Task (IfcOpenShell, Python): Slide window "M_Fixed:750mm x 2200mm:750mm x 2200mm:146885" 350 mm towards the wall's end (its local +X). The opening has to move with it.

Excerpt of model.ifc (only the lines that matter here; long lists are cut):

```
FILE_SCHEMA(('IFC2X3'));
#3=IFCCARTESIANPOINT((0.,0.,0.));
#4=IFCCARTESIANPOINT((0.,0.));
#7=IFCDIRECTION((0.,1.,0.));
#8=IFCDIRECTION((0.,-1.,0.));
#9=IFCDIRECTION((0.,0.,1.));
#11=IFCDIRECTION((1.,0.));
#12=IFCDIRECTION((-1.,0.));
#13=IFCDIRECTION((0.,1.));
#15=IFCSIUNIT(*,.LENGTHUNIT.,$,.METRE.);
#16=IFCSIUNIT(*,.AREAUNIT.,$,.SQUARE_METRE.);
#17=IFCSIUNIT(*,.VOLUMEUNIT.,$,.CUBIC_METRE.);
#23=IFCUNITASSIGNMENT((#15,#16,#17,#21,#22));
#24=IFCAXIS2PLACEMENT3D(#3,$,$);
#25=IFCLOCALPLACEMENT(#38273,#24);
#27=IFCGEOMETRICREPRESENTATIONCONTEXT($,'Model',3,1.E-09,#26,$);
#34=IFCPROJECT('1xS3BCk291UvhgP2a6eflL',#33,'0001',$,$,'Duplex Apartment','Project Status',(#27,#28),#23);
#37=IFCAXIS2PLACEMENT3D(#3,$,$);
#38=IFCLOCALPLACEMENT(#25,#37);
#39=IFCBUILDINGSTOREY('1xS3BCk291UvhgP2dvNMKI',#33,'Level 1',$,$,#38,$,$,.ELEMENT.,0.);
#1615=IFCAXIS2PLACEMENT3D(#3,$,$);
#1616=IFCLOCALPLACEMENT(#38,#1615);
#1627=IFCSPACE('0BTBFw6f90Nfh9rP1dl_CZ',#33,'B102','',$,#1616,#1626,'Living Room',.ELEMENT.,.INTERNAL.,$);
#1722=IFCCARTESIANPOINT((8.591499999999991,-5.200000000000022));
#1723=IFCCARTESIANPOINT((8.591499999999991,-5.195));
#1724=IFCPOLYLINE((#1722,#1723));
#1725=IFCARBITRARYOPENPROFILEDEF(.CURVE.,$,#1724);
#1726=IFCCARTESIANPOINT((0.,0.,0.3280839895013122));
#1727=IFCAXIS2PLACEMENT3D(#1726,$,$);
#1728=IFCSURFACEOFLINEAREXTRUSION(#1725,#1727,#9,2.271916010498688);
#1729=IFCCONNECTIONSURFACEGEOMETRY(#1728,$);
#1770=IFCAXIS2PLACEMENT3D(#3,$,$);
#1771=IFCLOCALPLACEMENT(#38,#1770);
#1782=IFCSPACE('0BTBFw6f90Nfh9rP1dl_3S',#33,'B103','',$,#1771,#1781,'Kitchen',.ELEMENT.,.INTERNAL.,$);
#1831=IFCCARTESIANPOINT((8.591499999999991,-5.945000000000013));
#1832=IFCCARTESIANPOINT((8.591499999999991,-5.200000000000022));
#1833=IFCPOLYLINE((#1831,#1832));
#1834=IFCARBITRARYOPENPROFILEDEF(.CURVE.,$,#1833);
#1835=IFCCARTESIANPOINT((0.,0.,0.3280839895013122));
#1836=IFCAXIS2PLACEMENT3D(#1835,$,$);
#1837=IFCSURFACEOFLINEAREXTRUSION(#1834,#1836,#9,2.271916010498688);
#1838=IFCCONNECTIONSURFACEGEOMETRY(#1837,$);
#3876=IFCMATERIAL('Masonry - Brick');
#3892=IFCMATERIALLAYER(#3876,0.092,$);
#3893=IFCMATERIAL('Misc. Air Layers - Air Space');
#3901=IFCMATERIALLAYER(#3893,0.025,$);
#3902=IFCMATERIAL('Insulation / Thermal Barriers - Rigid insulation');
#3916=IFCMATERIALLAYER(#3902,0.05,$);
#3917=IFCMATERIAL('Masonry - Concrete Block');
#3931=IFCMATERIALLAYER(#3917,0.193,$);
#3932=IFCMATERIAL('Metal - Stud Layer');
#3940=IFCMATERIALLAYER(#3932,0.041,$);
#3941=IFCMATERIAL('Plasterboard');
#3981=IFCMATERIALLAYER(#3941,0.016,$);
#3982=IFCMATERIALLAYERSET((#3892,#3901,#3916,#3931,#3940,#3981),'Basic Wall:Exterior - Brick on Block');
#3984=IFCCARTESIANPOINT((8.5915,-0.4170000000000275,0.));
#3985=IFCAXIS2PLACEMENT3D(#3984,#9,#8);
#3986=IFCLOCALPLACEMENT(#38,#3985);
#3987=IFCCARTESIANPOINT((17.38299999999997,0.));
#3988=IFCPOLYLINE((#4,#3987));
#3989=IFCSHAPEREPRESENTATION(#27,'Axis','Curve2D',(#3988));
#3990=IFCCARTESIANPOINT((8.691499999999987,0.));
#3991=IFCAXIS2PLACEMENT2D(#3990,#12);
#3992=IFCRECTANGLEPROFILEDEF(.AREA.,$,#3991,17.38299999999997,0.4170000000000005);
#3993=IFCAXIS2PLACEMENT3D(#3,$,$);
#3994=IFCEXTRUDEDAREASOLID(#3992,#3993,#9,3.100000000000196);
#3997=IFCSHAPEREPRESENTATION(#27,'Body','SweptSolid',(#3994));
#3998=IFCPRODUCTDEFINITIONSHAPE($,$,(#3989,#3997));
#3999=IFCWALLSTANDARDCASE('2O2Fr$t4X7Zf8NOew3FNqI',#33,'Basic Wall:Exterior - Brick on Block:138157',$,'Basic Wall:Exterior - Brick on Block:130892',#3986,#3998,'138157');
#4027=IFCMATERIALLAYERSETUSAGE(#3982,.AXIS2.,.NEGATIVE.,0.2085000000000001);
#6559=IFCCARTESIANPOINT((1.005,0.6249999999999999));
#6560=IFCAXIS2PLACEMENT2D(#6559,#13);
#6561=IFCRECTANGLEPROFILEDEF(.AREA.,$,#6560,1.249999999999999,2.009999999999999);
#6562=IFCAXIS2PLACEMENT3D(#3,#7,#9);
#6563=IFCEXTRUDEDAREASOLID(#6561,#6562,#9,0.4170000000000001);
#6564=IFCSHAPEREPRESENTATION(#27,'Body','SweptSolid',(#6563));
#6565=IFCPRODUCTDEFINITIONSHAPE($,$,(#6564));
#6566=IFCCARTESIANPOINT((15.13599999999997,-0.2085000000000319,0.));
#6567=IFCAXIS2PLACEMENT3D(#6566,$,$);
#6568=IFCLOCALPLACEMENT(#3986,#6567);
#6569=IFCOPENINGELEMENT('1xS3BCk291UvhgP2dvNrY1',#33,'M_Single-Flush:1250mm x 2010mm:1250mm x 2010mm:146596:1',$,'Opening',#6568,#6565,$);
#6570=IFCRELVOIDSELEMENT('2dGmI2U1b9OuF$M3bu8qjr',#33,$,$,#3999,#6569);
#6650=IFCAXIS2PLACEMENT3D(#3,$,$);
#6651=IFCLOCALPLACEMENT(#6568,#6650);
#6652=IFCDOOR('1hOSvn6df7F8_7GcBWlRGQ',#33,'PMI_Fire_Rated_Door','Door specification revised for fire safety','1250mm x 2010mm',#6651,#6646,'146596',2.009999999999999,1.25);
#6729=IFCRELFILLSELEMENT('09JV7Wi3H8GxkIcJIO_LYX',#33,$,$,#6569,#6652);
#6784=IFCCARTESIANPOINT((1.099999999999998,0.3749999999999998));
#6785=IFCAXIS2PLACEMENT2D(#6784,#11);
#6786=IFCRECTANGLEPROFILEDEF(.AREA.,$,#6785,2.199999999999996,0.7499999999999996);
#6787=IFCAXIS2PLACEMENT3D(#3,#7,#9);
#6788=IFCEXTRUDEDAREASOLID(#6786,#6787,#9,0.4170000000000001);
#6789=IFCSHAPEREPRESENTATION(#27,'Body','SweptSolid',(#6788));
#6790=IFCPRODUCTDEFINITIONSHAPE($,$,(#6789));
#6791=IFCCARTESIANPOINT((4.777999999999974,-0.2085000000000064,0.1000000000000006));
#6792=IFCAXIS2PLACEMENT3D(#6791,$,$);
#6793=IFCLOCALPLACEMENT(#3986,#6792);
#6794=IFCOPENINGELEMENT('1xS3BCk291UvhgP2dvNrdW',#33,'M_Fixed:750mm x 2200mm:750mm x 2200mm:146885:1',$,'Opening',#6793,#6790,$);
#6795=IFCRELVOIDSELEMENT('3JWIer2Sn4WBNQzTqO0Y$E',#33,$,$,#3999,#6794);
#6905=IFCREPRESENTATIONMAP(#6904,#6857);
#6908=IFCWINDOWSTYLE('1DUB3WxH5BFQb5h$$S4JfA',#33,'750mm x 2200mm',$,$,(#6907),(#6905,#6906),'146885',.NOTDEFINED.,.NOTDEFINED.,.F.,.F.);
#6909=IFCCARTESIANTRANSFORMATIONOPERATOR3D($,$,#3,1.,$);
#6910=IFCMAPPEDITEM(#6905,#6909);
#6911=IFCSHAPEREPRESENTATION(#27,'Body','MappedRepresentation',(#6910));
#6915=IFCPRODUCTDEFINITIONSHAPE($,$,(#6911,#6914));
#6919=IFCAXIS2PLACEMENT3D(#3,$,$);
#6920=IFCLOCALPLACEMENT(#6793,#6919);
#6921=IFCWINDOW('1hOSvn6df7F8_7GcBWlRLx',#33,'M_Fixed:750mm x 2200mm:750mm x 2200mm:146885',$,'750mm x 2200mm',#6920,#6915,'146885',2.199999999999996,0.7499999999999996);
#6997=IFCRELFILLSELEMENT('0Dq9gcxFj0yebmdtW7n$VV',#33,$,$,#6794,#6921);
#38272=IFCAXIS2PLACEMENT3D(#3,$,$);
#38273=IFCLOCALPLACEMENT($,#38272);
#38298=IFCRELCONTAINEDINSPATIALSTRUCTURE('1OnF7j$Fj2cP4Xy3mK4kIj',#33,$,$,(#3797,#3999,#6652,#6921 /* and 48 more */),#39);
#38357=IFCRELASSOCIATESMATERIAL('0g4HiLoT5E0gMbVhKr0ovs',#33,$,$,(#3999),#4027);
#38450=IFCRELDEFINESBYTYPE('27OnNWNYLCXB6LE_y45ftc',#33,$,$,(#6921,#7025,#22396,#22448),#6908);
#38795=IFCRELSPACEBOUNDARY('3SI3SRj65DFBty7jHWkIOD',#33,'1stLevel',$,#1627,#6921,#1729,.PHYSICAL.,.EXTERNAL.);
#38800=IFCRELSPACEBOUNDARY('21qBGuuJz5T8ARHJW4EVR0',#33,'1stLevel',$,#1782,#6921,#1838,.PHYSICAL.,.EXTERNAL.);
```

```python
import numpy as np
import ifcopenshell
import ifcopenshell.api.geometry
import ifcopenshell.util.placement

model = ifcopenshell.open("model.ifc")

window = model.by_id(6921)
opening = window.FillsVoids[0].RelatingOpeningElement
wall = opening.VoidsElements[0].RelatingBuildingElement

wall_matrix = ifcopenshell.util.placement.get_local_placement(wall.ObjectPlacement)
shift = wall_matrix[:3, 0] * 0.35
before = ifcopenshell.util.placement.get_local_placement(window.ObjectPlacement)[:3, 3].copy()

# The window is placed relative to its opening, so it follows when the opening moves.
matrix = ifcopenshell.util.placement.get_local_placement(opening.ObjectPlacement)
matrix[:3, 3] += shift
ifcopenshell.api.geometry.edit_object_placement(
    model, product=opening, matrix=matrix, is_si=False, should_transform_children=True
)

# Space boundary surfaces are stored in each space's coordinates; move them too.
for rel in window.ProvidesBoundaries:
    if not rel.ConnectionGeometry:
        continue
    surface = rel.ConnectionGeometry.SurfaceOnRelatingElement
    space_matrix = ifcopenshell.util.placement.get_local_placement(rel.RelatingSpace.ObjectPlacement)
    point = np.array(surface.Position.Location.Coordinates) + space_matrix[:3, :3].T @ shift
    surface.Position = model.createIfcAxis2Placement3D(
        model.createIfcCartesianPoint(point.tolist()), surface.Position.Axis, surface.Position.RefDirection
    )

after = ifcopenshell.util.placement.get_local_placement(window.ObjectPlacement)[:3, 3]
print("window moved by", (after - before).round(3) + 0.0)

model.write("model-out.ifc")
```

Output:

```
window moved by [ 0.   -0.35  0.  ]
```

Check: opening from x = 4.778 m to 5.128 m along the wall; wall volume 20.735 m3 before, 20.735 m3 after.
